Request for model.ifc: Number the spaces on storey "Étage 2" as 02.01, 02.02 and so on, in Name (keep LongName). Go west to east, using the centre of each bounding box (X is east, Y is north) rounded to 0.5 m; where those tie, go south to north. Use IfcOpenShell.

First a look at what the model holds.

```python
import ifcopenshell
import ifcopenshell.util.element
import ifcopenshell.util.placement

model = ifcopenshell.open("model.ifc")
print(model.schema)
storey = next(s for s in model.by_type("IfcBuildingStorey") if s.Name == "Étage 2")
spaces = [e for e in ifcopenshell.util.element.get_decomposition(storey) if e.is_a("IfcSpace")]
for e in sorted(spaces, key=lambda e: e.id()):
    origin = ifcopenshell.util.placement.get_local_placement(e.ObjectPlacement)[:3, 3]
    print(e.id(), e.Name, e.LongName, origin.round(2) + 0.0, sep=" | ")
```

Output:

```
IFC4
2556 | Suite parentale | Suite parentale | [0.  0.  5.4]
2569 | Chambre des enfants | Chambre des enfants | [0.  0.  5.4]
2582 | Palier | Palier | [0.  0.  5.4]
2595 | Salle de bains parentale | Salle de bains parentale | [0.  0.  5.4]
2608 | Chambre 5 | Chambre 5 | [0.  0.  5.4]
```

```python
import ifcopenshell
import ifcopenshell.geom
import ifcopenshell.util.element
import ifcopenshell.util.shape

model = ifcopenshell.open("model.ifc")
settings = ifcopenshell.geom.settings()
settings.set("use-world-coords", True)


def centre(element):
    shape = ifcopenshell.geom.create_shape(settings, element)
    return ifcopenshell.util.shape.get_bbox_centroid(shape.geometry)


storey = next(s for s in model.by_type("IfcBuildingStorey") if s.Name == "Étage 2")
spaces = [e for e in ifcopenshell.util.element.get_decomposition(storey) if e.is_a("IfcSpace")]

# Insertion points can sit at a corner or the storey origin, so sort by the geometry (in metres).
centres = {e: centre(e) for e in spaces}
spaces.sort(key=lambda e: (round(centres[e][0] / 0.5), centres[e][1]))

for i, e in enumerate(spaces, start=1):
    number = f"02.{i:02d}"
    e.Name = number
    print(e.id(), number)

model.write("model_updated.ifc")
```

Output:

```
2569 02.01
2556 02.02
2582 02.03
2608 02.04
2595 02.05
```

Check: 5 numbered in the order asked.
